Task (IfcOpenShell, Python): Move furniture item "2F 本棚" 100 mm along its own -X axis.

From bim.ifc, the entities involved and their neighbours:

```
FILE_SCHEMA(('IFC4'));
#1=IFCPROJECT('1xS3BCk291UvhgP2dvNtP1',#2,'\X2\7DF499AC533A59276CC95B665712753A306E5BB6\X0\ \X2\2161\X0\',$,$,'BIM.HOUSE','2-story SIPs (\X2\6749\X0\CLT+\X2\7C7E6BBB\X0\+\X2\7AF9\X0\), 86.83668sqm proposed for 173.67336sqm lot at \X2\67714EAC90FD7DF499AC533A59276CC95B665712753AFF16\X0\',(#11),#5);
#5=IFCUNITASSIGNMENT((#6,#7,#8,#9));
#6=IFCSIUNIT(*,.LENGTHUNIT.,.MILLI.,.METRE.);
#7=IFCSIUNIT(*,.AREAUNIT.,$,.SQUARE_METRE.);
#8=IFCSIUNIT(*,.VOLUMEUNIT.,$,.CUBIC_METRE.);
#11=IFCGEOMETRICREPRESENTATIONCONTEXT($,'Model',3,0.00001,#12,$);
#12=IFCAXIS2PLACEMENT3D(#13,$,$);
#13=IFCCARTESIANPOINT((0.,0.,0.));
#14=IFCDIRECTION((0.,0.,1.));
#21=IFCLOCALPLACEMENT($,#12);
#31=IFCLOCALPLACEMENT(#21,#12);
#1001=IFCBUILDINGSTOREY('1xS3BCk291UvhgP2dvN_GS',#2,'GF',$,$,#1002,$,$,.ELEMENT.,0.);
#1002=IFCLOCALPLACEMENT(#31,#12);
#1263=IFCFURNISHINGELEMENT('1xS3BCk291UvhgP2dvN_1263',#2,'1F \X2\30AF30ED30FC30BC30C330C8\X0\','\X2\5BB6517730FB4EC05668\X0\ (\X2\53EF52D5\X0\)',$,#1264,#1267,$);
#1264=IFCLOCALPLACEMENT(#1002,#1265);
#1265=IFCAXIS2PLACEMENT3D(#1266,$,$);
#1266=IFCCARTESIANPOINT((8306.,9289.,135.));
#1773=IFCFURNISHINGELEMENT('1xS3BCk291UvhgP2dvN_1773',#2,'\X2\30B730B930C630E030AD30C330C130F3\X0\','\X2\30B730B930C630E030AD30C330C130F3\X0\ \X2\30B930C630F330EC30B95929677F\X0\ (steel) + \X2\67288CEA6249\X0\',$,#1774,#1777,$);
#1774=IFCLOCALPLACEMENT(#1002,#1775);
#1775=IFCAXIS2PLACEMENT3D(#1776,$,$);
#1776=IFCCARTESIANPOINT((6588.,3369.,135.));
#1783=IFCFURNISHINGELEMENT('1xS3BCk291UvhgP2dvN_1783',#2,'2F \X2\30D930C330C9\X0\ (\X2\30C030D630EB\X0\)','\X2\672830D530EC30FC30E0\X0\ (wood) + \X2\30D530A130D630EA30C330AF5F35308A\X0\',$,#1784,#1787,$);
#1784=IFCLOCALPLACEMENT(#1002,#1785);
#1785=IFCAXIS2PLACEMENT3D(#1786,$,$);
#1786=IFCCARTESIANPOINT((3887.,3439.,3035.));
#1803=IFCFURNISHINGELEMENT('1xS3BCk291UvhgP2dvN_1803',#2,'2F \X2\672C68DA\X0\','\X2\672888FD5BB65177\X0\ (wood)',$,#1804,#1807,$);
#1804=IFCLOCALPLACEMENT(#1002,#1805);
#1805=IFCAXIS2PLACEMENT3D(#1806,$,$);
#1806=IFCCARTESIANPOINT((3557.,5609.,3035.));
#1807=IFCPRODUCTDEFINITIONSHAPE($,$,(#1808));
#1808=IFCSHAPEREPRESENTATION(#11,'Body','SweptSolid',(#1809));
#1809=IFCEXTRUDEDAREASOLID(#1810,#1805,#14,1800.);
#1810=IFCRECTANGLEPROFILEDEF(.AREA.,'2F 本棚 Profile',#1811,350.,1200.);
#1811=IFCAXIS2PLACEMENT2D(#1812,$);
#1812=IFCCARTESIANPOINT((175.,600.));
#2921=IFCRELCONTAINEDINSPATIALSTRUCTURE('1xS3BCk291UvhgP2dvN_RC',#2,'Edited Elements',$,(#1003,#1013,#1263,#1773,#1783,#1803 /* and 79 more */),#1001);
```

```python
import ifcopenshell
import ifcopenshell.api.geometry
import ifcopenshell.util.placement

model = ifcopenshell.open("bim.ifc")

item = model.by_id(1803)
matrix = ifcopenshell.util.placement.get_local_placement(item.ObjectPlacement)
matrix[:3, 3] -= matrix[:3, 0] * 100.0
ifcopenshell.api.geometry.edit_object_placement(model, product=item, matrix=matrix, is_si=False)

print(ifcopenshell.util.placement.get_local_placement(item.ObjectPlacement).round(3) + 0.0)

model.write("bim_edited.ifc")
```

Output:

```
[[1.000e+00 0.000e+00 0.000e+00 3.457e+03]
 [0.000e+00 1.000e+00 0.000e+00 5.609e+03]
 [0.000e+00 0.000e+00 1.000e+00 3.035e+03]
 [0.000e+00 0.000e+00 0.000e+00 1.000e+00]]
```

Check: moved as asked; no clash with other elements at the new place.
